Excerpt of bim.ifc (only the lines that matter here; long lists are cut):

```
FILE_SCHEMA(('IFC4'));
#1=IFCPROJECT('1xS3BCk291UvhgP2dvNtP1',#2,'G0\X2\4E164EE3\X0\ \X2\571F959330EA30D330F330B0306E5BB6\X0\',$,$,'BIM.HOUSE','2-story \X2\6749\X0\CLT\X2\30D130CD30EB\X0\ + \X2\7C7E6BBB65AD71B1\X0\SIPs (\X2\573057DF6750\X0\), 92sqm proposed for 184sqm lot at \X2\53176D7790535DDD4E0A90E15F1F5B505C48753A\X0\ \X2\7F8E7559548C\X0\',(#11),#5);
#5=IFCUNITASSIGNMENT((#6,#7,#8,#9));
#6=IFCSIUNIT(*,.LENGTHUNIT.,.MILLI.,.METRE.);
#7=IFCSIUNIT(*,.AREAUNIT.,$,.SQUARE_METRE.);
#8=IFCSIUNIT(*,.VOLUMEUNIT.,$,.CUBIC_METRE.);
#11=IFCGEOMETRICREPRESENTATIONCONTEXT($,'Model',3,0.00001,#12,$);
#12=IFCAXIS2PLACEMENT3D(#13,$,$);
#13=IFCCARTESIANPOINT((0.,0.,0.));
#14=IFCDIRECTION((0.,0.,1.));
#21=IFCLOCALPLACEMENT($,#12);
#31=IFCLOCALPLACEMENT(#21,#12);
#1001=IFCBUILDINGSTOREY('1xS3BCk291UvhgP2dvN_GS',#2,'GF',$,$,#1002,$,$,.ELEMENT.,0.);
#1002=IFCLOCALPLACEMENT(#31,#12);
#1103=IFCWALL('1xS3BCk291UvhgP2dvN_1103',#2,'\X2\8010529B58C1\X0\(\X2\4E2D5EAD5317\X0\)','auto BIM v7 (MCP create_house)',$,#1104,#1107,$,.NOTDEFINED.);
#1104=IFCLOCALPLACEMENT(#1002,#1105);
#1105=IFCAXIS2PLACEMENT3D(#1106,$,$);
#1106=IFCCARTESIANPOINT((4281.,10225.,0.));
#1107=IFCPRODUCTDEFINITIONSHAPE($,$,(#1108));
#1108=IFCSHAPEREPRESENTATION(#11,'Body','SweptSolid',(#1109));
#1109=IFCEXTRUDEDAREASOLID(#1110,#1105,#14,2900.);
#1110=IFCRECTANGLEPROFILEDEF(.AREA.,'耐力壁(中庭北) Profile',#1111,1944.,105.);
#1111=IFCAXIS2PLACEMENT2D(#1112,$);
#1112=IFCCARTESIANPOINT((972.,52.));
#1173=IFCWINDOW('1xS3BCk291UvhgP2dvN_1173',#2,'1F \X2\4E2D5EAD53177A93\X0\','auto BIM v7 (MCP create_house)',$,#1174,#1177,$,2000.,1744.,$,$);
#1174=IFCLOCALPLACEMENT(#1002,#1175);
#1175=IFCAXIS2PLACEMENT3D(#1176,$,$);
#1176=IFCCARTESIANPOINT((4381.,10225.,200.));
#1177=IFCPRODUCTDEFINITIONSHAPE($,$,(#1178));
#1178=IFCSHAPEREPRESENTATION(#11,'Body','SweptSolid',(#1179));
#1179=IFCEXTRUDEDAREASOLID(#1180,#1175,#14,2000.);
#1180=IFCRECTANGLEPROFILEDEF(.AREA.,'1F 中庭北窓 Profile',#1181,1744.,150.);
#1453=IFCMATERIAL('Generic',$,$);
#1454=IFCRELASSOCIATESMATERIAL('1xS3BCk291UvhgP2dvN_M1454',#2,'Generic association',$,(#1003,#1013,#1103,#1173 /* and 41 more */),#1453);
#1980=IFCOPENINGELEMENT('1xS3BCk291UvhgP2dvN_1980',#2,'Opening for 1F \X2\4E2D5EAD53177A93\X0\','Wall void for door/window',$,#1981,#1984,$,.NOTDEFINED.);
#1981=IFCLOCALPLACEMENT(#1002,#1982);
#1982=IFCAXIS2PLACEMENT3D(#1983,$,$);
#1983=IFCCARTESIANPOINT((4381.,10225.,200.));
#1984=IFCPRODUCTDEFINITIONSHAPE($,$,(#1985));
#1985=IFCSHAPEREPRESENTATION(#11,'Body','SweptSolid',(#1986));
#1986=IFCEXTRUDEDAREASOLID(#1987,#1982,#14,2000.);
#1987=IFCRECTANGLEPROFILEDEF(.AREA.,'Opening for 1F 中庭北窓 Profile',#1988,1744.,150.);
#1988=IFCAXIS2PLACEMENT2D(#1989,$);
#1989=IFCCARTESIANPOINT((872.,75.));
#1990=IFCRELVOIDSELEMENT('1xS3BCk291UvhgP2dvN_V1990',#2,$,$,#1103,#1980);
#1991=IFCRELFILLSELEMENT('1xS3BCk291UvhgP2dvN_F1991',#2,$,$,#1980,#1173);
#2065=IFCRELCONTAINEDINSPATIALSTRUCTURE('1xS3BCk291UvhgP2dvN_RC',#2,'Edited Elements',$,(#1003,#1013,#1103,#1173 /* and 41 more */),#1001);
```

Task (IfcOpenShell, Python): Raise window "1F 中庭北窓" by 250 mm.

```python
import numpy as np
import ifcopenshell
import ifcopenshell.api.geometry
import ifcopenshell.util.placement
import ifcopenshell.util.unit

model = ifcopenshell.open("bim.ifc")
unit_scale = ifcopenshell.util.unit.calculate_unit_scale(model)

window = model.by_guid("1xS3BCk291UvhgP2dvN_1173")
opening = window.FillsVoids[0].RelatingOpeningElement
dz = 250.0

shift = np.array([0.0, 0.0, dz])
# The window is not placed relative to its opening, so move both.
for product in (opening, window):
    matrix = ifcopenshell.util.placement.get_local_placement(product.ObjectPlacement)
    matrix[:3, 3] += shift
    ifcopenshell.api.geometry.edit_object_placement(model, product=product, matrix=matrix, is_si=False)

print(f"moved by {dz * unit_scale:+.3f} m")

model.write("bim_updated.ifc")
```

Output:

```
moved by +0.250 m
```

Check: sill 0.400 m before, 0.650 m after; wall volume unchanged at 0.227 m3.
